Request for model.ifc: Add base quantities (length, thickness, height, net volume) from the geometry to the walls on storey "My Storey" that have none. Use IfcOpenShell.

First a look at what the model holds.

```python
import ifcopenshell
import ifcopenshell.util.element
import ifcopenshell.util.unit

model = ifcopenshell.open("model.ifc")
print(model.schema)
for unit_type in ("LENGTHUNIT", "AREAUNIT", "VOLUMEUNIT"):
    print(unit_type, ifcopenshell.util.unit.calculate_unit_scale(model, unit_type))
storey = next(s for s in model.by_type("IfcBuildingStorey") if s.Name == "My Storey")
walls = [e for e in ifcopenshell.util.element.get_decomposition(storey) if e.is_a("IfcWall")]
for e in sorted(walls, key=lambda e: e.id()):
    print(e.id(), e.is_a(), e.Name, list(ifcopenshell.util.element.get_psets(e, qtos_only=True)), sep=" | ")
```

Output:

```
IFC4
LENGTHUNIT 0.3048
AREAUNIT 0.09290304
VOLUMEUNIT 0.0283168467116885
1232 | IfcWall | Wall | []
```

```python
import ifcopenshell
import ifcopenshell.api.pset
import ifcopenshell.geom
import ifcopenshell.util.element
import ifcopenshell.util.shape
import ifcopenshell.util.unit

model = ifcopenshell.open("model.ifc")
unit_scale = ifcopenshell.util.unit.calculate_unit_scale(model)
volume_scale = ifcopenshell.util.unit.calculate_unit_scale(model, "VOLUMEUNIT")
settings = ifcopenshell.geom.settings()

storey = next(s for s in model.by_type("IfcBuildingStorey") if s.Name == "My Storey")
walls = [e for e in ifcopenshell.util.element.get_decomposition(storey) if e.is_a("IfcWall")]

for e in sorted(walls, key=lambda e: e.id()):
    if ifcopenshell.util.element.get_psets(e, qtos_only=True, should_inherit=False):
        continue
    # Geometry comes back in metres, in the element's own axes.
    shape = ifcopenshell.geom.create_shape(settings, e)
    values = {
        "Length": ifcopenshell.util.shape.get_x(shape.geometry) / unit_scale,
        "Width": ifcopenshell.util.shape.get_y(shape.geometry) / unit_scale,
        "Height": ifcopenshell.util.shape.get_z(shape.geometry) / unit_scale,
        "NetVolume": ifcopenshell.util.shape.get_volume(shape.geometry) / volume_scale,
    }
    qto = ifcopenshell.api.pset.add_qto(model, product=e, name="Qto_WallBaseQuantities")
    ifcopenshell.api.pset.edit_qto(model, qto=qto, properties=values)
    print(e.id(), {k: round(v, 3) for k, v in values.items()})

model.write("model_rev.ifc")
```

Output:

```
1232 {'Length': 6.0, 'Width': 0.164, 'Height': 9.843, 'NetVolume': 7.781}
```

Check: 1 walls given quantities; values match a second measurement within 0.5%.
